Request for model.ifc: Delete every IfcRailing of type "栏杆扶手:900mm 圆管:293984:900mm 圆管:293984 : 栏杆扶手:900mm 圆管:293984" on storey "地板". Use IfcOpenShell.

First a look at what the model holds.

```python
import ifcopenshell
import ifcopenshell.util.element

model = ifcopenshell.open("model.ifc")
print(model.schema)
storey = next(s for s in model.by_type("IfcBuildingStorey") if s.Name == "地板")
railings = [e for e in ifcopenshell.util.element.get_decomposition(storey) if e.is_a("IfcRailing")]
seen = {}
for e in railings:
    element_type = ifcopenshell.util.element.get_type(e)
    name = element_type.Name if element_type not in (None, e) else None
    seen[name] = seen.get(name, 0) + 1
for name, count in sorted(seen.items(), key=str):
    print(count, "x", name)
```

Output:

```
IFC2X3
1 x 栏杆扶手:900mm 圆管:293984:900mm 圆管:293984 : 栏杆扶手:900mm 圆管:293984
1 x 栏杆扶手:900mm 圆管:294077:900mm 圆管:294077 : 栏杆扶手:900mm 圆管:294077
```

```python
import ifcopenshell
import ifcopenshell.api.root
import ifcopenshell.util.element

model = ifcopenshell.open("model.ifc")

storey = next(s for s in model.by_type("IfcBuildingStorey") if s.Name == "地板")
railings = [e for e in ifcopenshell.util.element.get_decomposition(storey) if e.is_a("IfcRailing")]
targets = [e for e in railings if (t := ifcopenshell.util.element.get_type(e)) not in (None, e) and t.Name == "栏杆扶手:900mm 圆管:293984:900mm 圆管:293984 : 栏杆扶手:900mm 圆管:293984"]

for e in targets:
    ifcopenshell.api.root.remove_product(model, product=e)
print(len(targets), "removed")

model.write("model-out.ifc")
```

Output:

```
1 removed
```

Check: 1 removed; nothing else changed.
